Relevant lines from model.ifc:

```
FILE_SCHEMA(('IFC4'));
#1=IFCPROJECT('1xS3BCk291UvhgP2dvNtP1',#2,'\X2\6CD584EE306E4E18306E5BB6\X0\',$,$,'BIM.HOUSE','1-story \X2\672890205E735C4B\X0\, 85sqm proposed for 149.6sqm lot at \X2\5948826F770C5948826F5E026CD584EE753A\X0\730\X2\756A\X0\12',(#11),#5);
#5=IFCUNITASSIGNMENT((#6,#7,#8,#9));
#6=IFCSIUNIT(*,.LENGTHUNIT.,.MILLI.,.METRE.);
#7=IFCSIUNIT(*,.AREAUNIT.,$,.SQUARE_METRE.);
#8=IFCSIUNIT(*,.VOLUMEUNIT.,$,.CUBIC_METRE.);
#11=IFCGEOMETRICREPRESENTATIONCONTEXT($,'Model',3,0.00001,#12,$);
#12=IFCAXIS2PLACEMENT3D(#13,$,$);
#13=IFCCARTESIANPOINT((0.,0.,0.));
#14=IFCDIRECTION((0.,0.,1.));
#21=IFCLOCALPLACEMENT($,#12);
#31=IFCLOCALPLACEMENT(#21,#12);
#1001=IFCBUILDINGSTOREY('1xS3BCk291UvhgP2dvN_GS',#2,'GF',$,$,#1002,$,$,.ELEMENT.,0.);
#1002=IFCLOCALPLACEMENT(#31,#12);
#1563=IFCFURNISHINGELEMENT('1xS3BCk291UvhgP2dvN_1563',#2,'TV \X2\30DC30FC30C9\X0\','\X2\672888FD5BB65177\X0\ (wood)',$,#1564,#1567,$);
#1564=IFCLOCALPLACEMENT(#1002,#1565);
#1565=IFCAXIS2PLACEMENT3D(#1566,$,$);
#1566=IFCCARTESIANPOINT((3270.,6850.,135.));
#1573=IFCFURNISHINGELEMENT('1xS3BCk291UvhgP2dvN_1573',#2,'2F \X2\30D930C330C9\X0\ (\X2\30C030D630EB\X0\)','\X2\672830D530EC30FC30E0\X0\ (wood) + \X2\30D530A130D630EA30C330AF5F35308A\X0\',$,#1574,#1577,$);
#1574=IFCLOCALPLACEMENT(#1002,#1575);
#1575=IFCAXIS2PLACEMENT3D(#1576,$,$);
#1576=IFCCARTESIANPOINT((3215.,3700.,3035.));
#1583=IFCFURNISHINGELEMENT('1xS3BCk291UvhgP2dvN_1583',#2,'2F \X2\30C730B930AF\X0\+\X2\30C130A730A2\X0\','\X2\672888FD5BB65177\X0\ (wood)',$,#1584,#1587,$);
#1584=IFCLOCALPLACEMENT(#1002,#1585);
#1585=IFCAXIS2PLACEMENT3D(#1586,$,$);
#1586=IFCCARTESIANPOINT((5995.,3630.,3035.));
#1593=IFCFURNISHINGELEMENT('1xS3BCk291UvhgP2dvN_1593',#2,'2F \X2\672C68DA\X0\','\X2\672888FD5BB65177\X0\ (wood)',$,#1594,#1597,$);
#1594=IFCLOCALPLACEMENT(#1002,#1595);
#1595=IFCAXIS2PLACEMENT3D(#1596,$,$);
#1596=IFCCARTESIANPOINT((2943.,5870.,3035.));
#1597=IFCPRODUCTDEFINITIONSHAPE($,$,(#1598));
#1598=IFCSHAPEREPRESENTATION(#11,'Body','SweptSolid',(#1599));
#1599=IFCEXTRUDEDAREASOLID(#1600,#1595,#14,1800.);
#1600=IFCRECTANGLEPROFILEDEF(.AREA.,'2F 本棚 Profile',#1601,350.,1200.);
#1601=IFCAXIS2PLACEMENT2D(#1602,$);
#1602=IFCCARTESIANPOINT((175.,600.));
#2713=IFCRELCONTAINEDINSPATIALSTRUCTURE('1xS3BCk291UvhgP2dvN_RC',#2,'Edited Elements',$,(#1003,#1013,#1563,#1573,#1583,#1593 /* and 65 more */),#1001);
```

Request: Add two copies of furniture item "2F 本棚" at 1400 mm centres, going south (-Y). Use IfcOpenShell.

```python
import numpy as np
import ifcopenshell
import ifcopenshell.api.geometry
import ifcopenshell.api.root
import ifcopenshell.util.element
import ifcopenshell.util.placement

model = ifcopenshell.open("model.ifc")


def reuse_history(source, copy):
    """copy_class also copies each property set's owner history, people and application; keep the originals."""
    for rel in copy.IsDefinedBy:
        if rel.is_a("IfcRelDefinesByProperties") and (history := rel.RelatingPropertyDefinition.OwnerHistory):
            rel.RelatingPropertyDefinition.OwnerHistory = source.OwnerHistory
            ifcopenshell.util.element.remove_deep2(model, history)


source = model.by_guid("1xS3BCk291UvhgP2dvN_1593")
base = ifcopenshell.util.placement.get_local_placement(source.ObjectPlacement)
step = np.array([0.0, -1.0, 0.0]) * 1400.0

for i in range(1, 3):
    copy = ifcopenshell.api.root.copy_class(model, product=source)
    copy.Representation = ifcopenshell.util.element.copy_deep(
        model, source.Representation, exclude=["IfcGeometricRepresentationContext", "IfcRepresentationMap"]
    )
    reuse_history(source, copy)
    matrix = base.copy()
    matrix[:3, 3] += i * step
    print("added at", matrix[:3, 3].round(3) + 0.0)
    ifcopenshell.api.geometry.edit_object_placement(model, product=copy, matrix=matrix, is_si=False)

model.write("model-out.ifc")
```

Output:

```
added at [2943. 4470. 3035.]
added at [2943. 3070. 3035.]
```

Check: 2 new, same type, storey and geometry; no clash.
